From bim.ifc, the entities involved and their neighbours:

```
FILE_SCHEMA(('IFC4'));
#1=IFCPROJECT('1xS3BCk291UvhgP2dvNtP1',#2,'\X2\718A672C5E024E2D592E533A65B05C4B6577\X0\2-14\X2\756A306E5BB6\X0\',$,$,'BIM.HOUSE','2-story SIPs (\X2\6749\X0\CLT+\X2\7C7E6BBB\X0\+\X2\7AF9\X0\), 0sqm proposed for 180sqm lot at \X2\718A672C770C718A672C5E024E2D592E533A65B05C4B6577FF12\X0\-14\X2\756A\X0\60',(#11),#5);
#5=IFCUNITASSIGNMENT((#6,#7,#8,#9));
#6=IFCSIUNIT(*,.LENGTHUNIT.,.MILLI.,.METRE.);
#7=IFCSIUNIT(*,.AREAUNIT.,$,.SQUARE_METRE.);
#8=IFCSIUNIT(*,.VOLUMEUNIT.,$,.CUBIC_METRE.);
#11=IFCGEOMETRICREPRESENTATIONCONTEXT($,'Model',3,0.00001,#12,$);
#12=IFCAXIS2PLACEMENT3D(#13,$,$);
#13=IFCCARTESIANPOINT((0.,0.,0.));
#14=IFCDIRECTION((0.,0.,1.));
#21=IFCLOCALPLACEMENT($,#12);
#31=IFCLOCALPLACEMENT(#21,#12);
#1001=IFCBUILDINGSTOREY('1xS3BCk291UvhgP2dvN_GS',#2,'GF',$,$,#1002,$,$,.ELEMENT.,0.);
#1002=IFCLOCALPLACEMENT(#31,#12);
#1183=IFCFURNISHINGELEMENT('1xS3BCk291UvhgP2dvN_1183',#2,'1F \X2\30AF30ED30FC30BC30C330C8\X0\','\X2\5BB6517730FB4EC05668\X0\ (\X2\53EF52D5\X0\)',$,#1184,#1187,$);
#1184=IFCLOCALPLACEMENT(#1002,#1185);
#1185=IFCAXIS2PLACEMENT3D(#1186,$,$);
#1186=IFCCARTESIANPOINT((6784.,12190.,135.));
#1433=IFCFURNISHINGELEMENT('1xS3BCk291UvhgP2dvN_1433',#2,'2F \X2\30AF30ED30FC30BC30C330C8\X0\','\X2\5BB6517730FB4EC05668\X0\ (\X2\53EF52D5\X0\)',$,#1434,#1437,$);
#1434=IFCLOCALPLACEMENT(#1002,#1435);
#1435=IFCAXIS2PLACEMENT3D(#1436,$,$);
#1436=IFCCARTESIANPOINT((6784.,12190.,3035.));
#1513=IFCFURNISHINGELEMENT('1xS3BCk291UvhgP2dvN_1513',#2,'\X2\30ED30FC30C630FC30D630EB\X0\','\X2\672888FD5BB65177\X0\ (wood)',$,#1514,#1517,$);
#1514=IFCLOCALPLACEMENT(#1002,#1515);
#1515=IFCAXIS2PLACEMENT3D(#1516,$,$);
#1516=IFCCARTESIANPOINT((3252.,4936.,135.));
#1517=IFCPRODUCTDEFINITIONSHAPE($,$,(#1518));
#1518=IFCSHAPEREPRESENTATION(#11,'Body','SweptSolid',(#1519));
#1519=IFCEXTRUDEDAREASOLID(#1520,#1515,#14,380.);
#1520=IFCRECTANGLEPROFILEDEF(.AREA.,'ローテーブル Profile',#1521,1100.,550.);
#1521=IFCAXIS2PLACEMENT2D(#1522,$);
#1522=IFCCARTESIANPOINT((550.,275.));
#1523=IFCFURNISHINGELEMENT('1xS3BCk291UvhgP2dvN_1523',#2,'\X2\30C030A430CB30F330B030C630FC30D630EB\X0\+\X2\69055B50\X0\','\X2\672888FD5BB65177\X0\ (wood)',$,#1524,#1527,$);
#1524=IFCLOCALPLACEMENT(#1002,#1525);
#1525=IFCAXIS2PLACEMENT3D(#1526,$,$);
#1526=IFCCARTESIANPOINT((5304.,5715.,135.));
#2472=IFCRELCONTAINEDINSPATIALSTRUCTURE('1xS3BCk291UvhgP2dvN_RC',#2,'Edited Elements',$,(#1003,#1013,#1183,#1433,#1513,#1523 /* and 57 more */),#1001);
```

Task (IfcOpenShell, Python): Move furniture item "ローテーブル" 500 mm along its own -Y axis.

```python
import ifcopenshell
import ifcopenshell.api.geometry
import ifcopenshell.util.placement
import ifcopenshell.util.unit

model = ifcopenshell.open("bim.ifc")
unit_scale = ifcopenshell.util.unit.calculate_unit_scale(model)

item = model.by_id(1513)
matrix = ifcopenshell.util.placement.get_local_placement(item.ObjectPlacement)
matrix[:3, 3] -= matrix[:3, 1] * 0.5 / unit_scale
ifcopenshell.api.geometry.edit_object_placement(model, product=item, matrix=matrix, is_si=False)

print(ifcopenshell.util.placement.get_local_placement(item.ObjectPlacement).round(3) + 0.0)

model.write("bim_edited.ifc")
```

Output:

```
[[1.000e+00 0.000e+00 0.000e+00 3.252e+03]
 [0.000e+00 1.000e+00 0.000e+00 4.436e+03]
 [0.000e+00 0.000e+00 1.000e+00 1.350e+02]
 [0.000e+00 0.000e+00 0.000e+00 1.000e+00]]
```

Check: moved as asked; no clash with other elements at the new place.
